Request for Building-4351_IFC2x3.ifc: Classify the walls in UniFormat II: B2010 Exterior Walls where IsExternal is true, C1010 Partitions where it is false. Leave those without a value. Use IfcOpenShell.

First a look at what the model holds.

```python
import ifcopenshell
import ifcopenshell.util.element

model = ifcopenshell.open("Building-4351_IFC2x3.ifc")
print(model.schema)
print("classifications:", [c.Name for c in model.by_type("IfcClassification")])
values = [ifcopenshell.util.element.get_pset(e, "Pset_WallCommon", "IsExternal") for e in model.by_type("IfcWall")]
for value in (True, False, None):
    print("IsExternal", value, values.count(value))
```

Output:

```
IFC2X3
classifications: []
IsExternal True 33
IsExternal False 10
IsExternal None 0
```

```python
import ifcopenshell
import ifcopenshell.api.classification
import ifcopenshell.util.element

model = ifcopenshell.open("Building-4351_IFC2x3.ifc")

# IFC2X3 requires Source and Edition and has no link from the project to the system.
system = model.create_entity("IfcClassification", Source="ASTM", Edition="E1557", Name="UniFormat II")

walls = model.by_type("IfcWall")
external = {e: ifcopenshell.util.element.get_pset(e, "Pset_WallCommon", "IsExternal") for e in walls}
for flag, code, name in ((True, "B2010", "Exterior Walls"), (False, "C1010", "Partitions")):
    products = [e for e in walls if external[e] is flag]
    ifcopenshell.api.classification.add_reference(
        model, products=products, classification=system, identification=code, name=name
    )
    print(code, len(products))

model.write("Building-4351_IFC2x3_edited.ifc")
```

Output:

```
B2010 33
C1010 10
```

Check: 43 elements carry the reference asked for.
